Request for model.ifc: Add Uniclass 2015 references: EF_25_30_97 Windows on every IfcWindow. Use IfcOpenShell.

First a look at what the model holds.

```python
import ifcopenshell

model = ifcopenshell.open("model.ifc")
print(model.schema)
print("classifications:", [c.Name for c in model.by_type("IfcClassification")])
for ifc_class in ("IfcDoor", "IfcRoof", "IfcStair", "IfcWall", "IfcWindow"):
    print(ifc_class, len(model.by_type(ifc_class)))
```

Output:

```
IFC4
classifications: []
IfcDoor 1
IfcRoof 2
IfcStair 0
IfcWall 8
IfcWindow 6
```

```python
import ifcopenshell
import ifcopenshell.api.classification

model = ifcopenshell.open("model.ifc")

system = ifcopenshell.api.classification.add_classification(model, classification="Uniclass 2015")

codes = {
    "IfcWindow": ("EF_25_30_97", "Windows"),
}
for ifc_class, (code, name) in codes.items():
    products = model.by_type(ifc_class)
    ifcopenshell.api.classification.add_reference(
        model, products=products, classification=system, identification=code, name=name
    )
    print(code, len(products))

model.write("model_v2.ifc")
```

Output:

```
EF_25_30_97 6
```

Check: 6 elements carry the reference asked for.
